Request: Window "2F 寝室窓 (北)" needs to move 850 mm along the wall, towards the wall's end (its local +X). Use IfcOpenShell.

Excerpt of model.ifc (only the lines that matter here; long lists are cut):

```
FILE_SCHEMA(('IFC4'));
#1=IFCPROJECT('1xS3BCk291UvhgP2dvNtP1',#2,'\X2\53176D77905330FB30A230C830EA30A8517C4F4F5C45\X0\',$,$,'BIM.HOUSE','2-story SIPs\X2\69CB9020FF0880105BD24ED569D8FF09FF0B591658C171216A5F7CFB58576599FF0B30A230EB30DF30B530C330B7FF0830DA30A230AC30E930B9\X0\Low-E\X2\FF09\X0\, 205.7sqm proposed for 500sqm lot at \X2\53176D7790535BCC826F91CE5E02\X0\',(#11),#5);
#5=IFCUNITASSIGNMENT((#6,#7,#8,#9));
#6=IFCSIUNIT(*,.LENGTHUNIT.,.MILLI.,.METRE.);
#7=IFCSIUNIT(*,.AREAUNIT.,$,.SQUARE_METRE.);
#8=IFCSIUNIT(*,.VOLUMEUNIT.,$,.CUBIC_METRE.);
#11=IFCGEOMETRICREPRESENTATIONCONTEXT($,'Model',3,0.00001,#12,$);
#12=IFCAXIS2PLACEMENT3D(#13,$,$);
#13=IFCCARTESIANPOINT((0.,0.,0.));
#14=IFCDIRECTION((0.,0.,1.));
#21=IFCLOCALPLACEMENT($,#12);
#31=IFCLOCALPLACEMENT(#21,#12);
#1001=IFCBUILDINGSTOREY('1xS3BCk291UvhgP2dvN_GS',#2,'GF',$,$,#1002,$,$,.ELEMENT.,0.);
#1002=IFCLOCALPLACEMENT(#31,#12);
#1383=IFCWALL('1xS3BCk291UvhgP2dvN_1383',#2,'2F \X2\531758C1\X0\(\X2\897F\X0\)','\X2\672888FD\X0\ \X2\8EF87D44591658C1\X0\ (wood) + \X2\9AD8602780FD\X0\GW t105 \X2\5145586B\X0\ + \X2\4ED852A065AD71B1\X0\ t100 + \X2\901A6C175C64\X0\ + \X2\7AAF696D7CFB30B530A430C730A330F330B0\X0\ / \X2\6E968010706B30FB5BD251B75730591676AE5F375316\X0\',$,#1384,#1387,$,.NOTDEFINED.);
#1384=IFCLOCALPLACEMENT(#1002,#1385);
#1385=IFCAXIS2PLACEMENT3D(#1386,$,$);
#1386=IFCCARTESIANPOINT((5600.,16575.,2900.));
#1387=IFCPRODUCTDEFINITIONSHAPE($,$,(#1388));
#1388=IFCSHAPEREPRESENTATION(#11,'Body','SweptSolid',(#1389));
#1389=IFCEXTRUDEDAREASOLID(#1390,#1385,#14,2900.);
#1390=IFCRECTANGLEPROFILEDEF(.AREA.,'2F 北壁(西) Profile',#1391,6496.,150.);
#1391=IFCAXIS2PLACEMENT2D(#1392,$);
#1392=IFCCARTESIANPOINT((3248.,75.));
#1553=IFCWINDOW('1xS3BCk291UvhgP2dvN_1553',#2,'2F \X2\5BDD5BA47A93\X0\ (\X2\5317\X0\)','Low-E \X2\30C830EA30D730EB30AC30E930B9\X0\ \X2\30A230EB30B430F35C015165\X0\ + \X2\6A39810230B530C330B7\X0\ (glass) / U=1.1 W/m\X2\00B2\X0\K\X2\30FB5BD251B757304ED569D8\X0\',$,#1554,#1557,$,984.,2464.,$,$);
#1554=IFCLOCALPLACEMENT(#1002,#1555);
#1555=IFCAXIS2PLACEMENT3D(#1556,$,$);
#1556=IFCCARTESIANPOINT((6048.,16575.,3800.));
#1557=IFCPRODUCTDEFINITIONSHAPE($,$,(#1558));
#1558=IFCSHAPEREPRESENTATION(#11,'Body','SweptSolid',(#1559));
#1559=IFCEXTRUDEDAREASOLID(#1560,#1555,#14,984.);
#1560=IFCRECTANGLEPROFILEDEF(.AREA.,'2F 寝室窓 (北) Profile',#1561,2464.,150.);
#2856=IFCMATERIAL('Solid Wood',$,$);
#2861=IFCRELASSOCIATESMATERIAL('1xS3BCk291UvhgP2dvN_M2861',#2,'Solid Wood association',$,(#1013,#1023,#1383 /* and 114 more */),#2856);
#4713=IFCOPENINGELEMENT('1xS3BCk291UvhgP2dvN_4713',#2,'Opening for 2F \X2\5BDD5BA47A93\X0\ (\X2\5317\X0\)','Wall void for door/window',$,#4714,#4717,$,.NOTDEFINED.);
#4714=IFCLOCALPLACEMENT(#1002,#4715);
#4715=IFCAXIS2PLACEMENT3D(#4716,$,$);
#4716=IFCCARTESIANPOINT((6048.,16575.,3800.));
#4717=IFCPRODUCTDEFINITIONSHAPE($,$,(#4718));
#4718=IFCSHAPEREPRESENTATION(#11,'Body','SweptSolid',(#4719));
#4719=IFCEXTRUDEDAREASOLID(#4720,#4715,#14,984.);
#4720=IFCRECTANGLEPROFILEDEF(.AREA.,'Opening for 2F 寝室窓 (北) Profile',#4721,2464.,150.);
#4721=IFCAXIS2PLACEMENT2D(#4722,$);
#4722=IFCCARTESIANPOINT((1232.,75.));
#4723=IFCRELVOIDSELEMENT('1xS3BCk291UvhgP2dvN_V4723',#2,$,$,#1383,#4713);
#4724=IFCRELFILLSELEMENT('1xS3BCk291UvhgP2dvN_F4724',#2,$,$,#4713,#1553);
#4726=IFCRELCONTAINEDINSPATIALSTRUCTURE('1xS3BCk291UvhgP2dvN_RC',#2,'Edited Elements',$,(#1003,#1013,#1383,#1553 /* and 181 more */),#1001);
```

```python
import ifcopenshell
import ifcopenshell.api.geometry
import ifcopenshell.util.placement
import ifcopenshell.util.unit

model = ifcopenshell.open("model.ifc")
unit_scale = ifcopenshell.util.unit.calculate_unit_scale(model)

window = model.by_guid("1xS3BCk291UvhgP2dvN_1553")
opening = window.FillsVoids[0].RelatingOpeningElement
wall = opening.VoidsElements[0].RelatingBuildingElement

wall_matrix = ifcopenshell.util.placement.get_local_placement(wall.ObjectPlacement)
shift = wall_matrix[:3, 0] * 0.85 / unit_scale
before = ifcopenshell.util.placement.get_local_placement(window.ObjectPlacement)[:3, 3].copy()

# The window is not placed relative to its opening, so move both.
for product in (opening, window):
    matrix = ifcopenshell.util.placement.get_local_placement(product.ObjectPlacement)
    matrix[:3, 3] += shift
    ifcopenshell.api.geometry.edit_object_placement(model, product=product, matrix=matrix, is_si=False)

after = ifcopenshell.util.placement.get_local_placement(window.ObjectPlacement)[:3, 3]
print("window moved by", (after - before).round(3) + 0.0)

model.write("model_edited.ifc")
```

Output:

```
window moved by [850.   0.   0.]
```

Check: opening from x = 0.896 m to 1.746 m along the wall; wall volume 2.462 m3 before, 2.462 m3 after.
